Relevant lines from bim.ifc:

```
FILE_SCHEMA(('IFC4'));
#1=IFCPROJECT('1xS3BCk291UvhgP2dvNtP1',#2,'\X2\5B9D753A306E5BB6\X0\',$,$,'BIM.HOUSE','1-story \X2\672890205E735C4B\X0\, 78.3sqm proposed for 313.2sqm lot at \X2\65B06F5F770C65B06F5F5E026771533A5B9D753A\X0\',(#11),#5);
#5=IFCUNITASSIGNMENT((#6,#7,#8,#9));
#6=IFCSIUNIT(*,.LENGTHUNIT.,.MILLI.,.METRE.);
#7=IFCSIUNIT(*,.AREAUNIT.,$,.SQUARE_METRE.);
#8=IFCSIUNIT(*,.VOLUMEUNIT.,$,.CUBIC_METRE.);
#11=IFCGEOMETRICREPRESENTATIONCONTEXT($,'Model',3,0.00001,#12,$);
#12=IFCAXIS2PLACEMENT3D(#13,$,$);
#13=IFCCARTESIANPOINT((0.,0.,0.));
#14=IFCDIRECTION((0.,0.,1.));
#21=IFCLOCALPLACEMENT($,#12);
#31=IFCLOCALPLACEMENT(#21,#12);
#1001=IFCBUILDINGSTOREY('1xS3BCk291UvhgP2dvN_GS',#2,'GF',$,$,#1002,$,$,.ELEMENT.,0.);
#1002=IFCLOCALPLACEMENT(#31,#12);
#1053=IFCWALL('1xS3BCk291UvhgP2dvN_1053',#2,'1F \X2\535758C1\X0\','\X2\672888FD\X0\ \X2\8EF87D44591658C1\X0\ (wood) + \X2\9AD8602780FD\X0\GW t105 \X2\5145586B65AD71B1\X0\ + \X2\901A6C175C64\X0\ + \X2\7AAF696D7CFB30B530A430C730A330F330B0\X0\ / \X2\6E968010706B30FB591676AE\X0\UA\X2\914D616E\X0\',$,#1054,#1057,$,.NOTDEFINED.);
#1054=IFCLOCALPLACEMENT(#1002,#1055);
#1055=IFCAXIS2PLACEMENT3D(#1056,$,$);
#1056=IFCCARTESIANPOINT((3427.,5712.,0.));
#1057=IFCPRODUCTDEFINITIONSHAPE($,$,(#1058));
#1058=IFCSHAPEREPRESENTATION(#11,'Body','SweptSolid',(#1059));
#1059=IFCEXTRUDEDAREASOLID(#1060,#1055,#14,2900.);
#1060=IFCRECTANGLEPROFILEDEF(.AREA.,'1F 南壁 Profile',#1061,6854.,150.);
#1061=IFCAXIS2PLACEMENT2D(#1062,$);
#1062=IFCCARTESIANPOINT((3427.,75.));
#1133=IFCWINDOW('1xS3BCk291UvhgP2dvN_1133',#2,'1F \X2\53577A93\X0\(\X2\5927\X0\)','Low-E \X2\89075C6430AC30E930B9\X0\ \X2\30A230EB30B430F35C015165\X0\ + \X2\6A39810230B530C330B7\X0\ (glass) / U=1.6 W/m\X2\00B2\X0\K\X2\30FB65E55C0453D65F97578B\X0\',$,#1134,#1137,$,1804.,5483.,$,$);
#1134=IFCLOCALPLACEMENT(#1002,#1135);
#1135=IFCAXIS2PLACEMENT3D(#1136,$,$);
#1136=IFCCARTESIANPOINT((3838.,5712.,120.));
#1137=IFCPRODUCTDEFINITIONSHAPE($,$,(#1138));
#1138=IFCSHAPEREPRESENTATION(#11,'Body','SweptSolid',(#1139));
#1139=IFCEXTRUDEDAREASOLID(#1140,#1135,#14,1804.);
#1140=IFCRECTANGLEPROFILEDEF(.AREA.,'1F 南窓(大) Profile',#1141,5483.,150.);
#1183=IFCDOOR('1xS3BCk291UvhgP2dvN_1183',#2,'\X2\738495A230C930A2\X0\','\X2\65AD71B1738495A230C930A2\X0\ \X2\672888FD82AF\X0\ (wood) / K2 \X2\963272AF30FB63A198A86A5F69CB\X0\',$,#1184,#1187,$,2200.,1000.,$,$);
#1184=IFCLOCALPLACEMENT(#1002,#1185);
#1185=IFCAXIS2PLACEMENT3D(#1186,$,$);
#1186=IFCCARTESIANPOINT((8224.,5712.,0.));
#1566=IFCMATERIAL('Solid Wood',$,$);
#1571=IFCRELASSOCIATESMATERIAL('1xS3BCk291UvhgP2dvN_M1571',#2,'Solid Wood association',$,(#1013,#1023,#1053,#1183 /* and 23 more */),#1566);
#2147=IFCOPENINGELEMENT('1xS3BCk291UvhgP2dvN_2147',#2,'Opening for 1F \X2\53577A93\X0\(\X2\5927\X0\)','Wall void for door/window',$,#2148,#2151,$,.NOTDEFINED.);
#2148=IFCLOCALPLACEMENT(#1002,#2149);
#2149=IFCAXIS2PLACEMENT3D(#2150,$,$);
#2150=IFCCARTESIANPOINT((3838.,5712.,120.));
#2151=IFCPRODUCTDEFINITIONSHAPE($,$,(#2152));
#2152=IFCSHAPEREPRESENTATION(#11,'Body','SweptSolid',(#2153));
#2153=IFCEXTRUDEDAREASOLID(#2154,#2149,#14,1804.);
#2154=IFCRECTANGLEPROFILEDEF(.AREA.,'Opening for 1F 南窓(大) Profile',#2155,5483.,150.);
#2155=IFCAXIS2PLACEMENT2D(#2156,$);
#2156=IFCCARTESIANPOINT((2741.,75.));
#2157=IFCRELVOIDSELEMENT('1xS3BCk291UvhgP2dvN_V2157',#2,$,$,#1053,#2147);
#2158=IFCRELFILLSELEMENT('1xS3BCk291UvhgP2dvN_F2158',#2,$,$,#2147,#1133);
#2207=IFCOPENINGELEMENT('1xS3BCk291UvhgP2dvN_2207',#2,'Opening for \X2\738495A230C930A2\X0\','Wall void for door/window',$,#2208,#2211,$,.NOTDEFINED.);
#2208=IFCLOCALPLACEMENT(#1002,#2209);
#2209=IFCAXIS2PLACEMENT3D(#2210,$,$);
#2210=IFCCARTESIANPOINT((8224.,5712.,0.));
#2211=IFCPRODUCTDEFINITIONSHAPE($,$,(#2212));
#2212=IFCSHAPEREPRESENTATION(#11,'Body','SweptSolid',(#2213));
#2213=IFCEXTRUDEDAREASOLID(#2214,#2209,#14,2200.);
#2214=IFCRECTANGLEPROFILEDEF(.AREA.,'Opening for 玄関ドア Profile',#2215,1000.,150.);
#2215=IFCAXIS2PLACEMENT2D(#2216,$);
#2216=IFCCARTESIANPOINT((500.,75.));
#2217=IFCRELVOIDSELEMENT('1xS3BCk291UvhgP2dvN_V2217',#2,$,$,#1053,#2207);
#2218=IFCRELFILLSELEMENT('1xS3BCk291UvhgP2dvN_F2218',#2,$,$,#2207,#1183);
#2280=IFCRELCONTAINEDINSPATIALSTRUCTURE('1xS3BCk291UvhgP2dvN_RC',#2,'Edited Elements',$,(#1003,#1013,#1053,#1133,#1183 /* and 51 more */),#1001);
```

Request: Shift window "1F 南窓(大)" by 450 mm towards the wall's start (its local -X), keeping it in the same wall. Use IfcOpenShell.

```python
import ifcopenshell
import ifcopenshell.api.geometry
import ifcopenshell.util.placement

model = ifcopenshell.open("bim.ifc")

window = model.by_guid("1xS3BCk291UvhgP2dvN_1133")
opening = window.FillsVoids[0].RelatingOpeningElement
wall = opening.VoidsElements[0].RelatingBuildingElement

wall_matrix = ifcopenshell.util.placement.get_local_placement(wall.ObjectPlacement)
shift = wall_matrix[:3, 0] * -450.0
before = ifcopenshell.util.placement.get_local_placement(window.ObjectPlacement)[:3, 3].copy()

# The window is not placed relative to its opening, so move both.
for product in (opening, window):
    matrix = ifcopenshell.util.placement.get_local_placement(product.ObjectPlacement)
    matrix[:3, 3] += shift
    ifcopenshell.api.geometry.edit_object_placement(model, product=product, matrix=matrix, is_si=False)

after = ifcopenshell.util.placement.get_local_placement(window.ObjectPlacement)[:3, 3]
print("window moved by", (after - before).round(3) + 0.0)

model.write("bim_updated.ifc")
```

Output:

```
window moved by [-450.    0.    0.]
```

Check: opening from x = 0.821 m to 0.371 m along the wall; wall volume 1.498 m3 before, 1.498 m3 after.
